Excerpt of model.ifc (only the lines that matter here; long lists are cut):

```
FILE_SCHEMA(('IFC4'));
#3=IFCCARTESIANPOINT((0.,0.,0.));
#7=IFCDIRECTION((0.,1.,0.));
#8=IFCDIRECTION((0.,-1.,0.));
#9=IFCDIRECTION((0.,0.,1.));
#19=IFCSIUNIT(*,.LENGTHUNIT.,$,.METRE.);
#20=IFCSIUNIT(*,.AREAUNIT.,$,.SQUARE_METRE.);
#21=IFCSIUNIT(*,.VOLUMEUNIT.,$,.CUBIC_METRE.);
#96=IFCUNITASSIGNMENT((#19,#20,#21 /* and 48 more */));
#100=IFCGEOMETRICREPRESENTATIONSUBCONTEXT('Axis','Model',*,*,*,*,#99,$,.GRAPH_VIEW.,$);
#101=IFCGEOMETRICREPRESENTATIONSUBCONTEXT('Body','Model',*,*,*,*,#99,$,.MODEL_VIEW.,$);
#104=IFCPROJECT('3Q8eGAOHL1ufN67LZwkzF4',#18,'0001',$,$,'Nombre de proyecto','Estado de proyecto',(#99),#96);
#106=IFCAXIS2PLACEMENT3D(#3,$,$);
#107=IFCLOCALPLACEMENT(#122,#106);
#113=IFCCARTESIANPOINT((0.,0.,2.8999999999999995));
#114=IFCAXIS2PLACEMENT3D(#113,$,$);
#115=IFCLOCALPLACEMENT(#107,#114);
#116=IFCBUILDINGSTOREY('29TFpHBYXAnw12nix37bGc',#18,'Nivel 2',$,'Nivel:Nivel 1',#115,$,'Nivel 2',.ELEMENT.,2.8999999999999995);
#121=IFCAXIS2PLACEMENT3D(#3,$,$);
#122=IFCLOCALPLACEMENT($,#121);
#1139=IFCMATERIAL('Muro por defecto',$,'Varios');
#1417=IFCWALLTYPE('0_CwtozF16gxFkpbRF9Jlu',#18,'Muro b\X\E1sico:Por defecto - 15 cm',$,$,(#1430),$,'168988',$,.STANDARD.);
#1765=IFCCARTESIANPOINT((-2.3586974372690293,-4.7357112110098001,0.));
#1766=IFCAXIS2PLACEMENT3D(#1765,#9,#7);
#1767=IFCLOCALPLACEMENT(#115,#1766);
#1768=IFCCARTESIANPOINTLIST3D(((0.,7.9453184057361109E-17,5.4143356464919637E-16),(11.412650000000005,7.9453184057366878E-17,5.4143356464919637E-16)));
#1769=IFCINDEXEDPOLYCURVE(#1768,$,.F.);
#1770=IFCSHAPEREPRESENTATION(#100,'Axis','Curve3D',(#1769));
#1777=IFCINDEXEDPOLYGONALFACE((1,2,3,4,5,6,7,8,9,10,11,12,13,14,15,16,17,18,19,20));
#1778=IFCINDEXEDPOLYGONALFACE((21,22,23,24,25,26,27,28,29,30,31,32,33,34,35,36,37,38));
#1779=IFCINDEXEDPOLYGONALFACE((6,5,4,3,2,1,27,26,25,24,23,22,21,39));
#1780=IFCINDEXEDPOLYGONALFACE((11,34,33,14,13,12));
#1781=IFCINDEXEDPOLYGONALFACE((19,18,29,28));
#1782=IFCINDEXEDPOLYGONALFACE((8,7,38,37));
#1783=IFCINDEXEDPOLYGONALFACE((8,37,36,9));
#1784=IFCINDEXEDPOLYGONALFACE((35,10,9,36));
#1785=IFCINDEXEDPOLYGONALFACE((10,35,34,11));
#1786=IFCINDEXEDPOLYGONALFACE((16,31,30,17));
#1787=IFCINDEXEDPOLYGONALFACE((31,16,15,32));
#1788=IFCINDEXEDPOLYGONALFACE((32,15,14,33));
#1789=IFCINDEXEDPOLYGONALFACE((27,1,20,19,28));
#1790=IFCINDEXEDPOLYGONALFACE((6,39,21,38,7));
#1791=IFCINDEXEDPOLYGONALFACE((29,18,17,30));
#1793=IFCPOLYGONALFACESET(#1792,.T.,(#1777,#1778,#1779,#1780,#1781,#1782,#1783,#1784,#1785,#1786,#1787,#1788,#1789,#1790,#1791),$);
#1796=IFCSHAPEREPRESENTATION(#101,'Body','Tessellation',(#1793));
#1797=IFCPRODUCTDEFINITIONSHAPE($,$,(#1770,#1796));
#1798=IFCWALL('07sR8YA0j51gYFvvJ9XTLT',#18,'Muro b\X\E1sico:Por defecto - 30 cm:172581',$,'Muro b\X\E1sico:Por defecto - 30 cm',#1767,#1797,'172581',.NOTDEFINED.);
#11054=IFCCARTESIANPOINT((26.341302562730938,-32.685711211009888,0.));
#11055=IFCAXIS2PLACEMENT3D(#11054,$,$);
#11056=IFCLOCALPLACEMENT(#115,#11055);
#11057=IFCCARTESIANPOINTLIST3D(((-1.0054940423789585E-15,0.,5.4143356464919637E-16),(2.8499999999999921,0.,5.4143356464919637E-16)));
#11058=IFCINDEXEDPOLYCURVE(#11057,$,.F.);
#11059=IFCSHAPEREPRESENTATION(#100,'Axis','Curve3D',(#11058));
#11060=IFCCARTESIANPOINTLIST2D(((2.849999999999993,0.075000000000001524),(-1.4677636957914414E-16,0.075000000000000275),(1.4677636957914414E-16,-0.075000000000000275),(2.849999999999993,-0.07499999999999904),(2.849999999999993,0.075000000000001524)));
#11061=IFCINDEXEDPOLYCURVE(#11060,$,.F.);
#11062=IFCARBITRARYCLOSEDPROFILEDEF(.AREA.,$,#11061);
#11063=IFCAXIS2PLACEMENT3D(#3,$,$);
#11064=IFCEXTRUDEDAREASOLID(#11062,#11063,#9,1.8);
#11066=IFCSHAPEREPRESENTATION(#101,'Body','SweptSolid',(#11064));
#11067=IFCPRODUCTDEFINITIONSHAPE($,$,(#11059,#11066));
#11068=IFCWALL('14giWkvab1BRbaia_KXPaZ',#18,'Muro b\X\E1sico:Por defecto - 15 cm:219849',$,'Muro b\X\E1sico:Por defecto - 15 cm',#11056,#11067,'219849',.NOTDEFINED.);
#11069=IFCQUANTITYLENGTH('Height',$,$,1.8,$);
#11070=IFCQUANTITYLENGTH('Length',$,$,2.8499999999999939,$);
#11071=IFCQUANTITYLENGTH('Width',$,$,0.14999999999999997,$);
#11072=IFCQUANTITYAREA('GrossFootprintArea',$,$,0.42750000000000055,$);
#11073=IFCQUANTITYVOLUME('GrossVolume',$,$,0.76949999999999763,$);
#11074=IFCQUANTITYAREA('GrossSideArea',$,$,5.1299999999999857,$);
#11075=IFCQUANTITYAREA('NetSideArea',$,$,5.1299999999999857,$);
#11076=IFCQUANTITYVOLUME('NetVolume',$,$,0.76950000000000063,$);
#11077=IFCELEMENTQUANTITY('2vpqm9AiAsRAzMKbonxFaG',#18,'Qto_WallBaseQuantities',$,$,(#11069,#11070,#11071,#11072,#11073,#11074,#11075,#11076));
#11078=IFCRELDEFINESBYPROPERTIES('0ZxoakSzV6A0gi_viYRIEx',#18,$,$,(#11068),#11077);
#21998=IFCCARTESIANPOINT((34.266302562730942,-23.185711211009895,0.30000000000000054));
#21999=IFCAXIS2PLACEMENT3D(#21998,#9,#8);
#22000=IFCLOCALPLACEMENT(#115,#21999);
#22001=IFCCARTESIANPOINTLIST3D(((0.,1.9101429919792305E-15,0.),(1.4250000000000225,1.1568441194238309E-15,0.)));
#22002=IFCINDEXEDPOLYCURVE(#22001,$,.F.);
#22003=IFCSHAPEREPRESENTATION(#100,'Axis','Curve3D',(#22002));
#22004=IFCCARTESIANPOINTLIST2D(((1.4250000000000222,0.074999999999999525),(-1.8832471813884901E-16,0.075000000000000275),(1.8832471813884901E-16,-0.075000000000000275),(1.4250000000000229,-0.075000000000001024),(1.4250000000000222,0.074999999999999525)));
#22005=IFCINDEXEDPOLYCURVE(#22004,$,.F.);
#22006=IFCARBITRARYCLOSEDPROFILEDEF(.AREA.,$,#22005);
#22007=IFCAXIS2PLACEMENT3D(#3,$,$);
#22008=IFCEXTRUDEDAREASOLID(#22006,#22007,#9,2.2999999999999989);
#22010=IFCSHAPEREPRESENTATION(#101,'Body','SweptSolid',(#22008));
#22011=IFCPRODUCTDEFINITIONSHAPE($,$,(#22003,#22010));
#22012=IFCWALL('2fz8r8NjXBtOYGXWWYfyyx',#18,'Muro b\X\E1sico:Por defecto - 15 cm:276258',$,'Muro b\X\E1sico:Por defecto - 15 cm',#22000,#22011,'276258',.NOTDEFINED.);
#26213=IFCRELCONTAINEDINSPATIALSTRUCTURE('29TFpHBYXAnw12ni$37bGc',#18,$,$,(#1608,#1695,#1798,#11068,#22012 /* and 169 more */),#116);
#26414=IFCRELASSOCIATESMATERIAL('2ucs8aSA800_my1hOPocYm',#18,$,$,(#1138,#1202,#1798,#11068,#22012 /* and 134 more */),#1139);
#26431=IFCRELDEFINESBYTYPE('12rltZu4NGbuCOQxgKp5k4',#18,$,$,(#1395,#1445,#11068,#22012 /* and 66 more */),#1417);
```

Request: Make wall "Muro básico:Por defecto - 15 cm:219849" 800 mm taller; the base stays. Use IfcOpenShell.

```python
import ifcopenshell
import ifcopenshell.api.pset
import ifcopenshell.geom
import ifcopenshell.util.element
import ifcopenshell.util.representation
import ifcopenshell.util.shape
import ifcopenshell.util.unit

model = ifcopenshell.open("model.ifc")
unit_scale = ifcopenshell.util.unit.calculate_unit_scale(model)
area_scale = ifcopenshell.util.unit.calculate_unit_scale(model, "AREAUNIT")
volume_scale = ifcopenshell.util.unit.calculate_unit_scale(model, "VOLUMEUNIT")
settings = ifcopenshell.geom.settings()


def volume(element):
    """Net volume in cubic metres, openings subtracted."""
    shape = ifcopenshell.geom.create_shape(settings, element)
    return ifcopenshell.util.shape.get_volume(shape.geometry)


wall = model.by_guid("14giWkvab1BRbaia_KXPaZ")
before = volume(wall)

body = ifcopenshell.util.representation.get_representation(wall, "Model", "Body")
solid = body.Items[0]
old_height = solid.Depth
solid.Depth += 0.8 / unit_scale
after = volume(wall)
thickness = 0.15  # wall thickness in metres

# Update the stored height, areas and volumes.
qto = model.by_id(ifcopenshell.util.element.get_pset(wall, "Qto_WallBaseQuantities", should_inherit=False)["id"])
ifcopenshell.api.pset.edit_qto(model, qto=qto, properties={
    "Height": solid.Depth,
    "GrossVolume": ifcopenshell.util.element.get_pset(wall, "Qto_WallBaseQuantities", "GrossVolume") * solid.Depth / old_height,
    "GrossSideArea": ifcopenshell.util.element.get_pset(wall, "Qto_WallBaseQuantities", "GrossSideArea") * solid.Depth / old_height,
    "NetSideArea": after / thickness / area_scale,
    "NetVolume": after / volume_scale,
})

print(f"height {old_height:g} -> {solid.Depth:g}, volume {before:.3f} -> {after:.3f} m3")

model.write("model-out.ifc")
```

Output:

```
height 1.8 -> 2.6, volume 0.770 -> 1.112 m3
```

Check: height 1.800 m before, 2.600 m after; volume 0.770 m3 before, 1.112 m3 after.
